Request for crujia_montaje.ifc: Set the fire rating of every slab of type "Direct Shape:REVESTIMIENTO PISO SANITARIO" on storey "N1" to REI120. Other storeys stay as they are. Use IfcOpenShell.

First a look at what the model holds.

```python
import ifcopenshell
import ifcopenshell.util.element

model = ifcopenshell.open("crujia_montaje.ifc")
print(model.schema)
storey = next(s for s in model.by_type("IfcBuildingStorey") if s.Name == "N1")
slabs = [e for e in ifcopenshell.util.element.get_decomposition(storey) if e.is_a("IfcSlab")]
seen = {}
for e in slabs:
    element_type = ifcopenshell.util.element.get_type(e)
    key = (element_type.Name if element_type != e and element_type else None, ifcopenshell.util.element.get_pset(e, "Pset_SlabCommon", "FireRating"))
    seen[key] = seen.get(key, 0) + 1
for (name, value), count in sorted(seen.items(), key=str):
    print(count, "x", name, "|", value)
```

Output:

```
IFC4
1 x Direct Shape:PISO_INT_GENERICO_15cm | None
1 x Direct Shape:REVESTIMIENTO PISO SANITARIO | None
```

```python
import ifcopenshell
import ifcopenshell.api.pset
import ifcopenshell.util.element

model = ifcopenshell.open("crujia_montaje.ifc")

storey = next(s for s in model.by_type("IfcBuildingStorey") if s.Name == "N1")
slabs = [e for e in ifcopenshell.util.element.get_decomposition(storey) if e.is_a("IfcSlab")]

count = 0
for e in slabs:
    element_type = ifcopenshell.util.element.get_type(e)
    if element_type in (None, e) or element_type.Name != "Direct Shape:REVESTIMIENTO PISO SANITARIO":
        continue
    # add_pset returns the element's existing set when there is one.
    pset = ifcopenshell.api.pset.add_pset(model, product=e, name="Pset_SlabCommon")
    ifcopenshell.api.pset.edit_pset(model, pset=pset, properties={"FireRating": "REI120"})
    count += 1

print(count, "slabs updated")

model.write("crujia_montaje_rev.ifc")
```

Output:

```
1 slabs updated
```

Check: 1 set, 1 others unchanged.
